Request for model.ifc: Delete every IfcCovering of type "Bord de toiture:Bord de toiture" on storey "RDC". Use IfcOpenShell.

First a look at what the model holds.

```python
import ifcopenshell
import ifcopenshell.util.element

model = ifcopenshell.open("model.ifc")
print(model.schema)
storey = next(s for s in model.by_type("IfcBuildingStorey") if s.Name == "RDC")
coverings = [e for e in ifcopenshell.util.element.get_decomposition(storey) if e.is_a("IfcCovering")]
seen = {}
for e in coverings:
    element_type = ifcopenshell.util.element.get_type(e)
    name = element_type.Name if element_type not in (None, e) else None
    seen[name] = seen.get(name, 0) + 1
for name, count in sorted(seen.items(), key=str):
    print(count, "x", name)
```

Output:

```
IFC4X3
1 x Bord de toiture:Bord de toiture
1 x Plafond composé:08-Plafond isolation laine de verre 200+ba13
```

```python
import ifcopenshell
import ifcopenshell.api.root
import ifcopenshell.util.element

model = ifcopenshell.open("model.ifc")

storey = next(s for s in model.by_type("IfcBuildingStorey") if s.Name == "RDC")
coverings = [e for e in ifcopenshell.util.element.get_decomposition(storey) if e.is_a("IfcCovering")]
targets = [e for e in coverings if (t := ifcopenshell.util.element.get_type(e)) not in (None, e) and t.Name == "Bord de toiture:Bord de toiture"]

for e in targets:
    ifcopenshell.api.root.remove_product(model, product=e)
print(len(targets), "removed")

model.write("model_updated.ifc")
```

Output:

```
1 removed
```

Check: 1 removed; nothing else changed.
